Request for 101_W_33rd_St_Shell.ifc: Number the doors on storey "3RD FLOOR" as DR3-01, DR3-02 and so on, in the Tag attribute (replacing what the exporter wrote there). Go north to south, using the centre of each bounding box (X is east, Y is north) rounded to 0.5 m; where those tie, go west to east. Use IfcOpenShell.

First a look at what the model holds.

```python
import ifcopenshell
import ifcopenshell.util.element
import ifcopenshell.util.placement

model = ifcopenshell.open("101_W_33rd_St_Shell.ifc")
print(model.schema)
storey = next(s for s in model.by_type("IfcBuildingStorey") if s.Name == "3RD FLOOR")
doors = [e for e in ifcopenshell.util.element.get_decomposition(storey) if e.is_a("IfcDoor")]
for e in sorted(doors, key=lambda e: e.id()):
    origin = ifcopenshell.util.placement.get_local_placement(e.ObjectPlacement)[:3, 3]
    print(e.id(), e.Tag, e.Name, origin.round(2) + 0.0, sep=" | ")
```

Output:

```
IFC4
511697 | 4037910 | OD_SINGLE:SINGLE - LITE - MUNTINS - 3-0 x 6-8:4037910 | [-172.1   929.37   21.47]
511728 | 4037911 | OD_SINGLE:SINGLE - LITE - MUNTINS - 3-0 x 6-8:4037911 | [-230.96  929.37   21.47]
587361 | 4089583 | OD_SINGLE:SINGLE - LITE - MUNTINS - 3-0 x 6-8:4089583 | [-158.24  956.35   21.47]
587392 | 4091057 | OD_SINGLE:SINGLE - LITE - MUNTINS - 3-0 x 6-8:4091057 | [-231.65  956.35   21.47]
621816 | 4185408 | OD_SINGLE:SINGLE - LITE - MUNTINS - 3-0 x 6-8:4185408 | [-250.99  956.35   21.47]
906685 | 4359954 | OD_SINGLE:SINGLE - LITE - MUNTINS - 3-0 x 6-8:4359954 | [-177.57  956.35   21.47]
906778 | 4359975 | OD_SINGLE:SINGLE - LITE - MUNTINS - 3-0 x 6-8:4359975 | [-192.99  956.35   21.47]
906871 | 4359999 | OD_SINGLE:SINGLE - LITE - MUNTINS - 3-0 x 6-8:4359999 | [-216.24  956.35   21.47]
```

```python
import ifcopenshell
import ifcopenshell.geom
import ifcopenshell.util.element
import ifcopenshell.util.shape

model = ifcopenshell.open("101_W_33rd_St_Shell.ifc")
settings = ifcopenshell.geom.settings()
settings.set("use-world-coords", True)


def centre(element):
    shape = ifcopenshell.geom.create_shape(settings, element)
    return ifcopenshell.util.shape.get_bbox_centroid(shape.geometry)


storey = next(s for s in model.by_type("IfcBuildingStorey") if s.Name == "3RD FLOOR")
doors = [e for e in ifcopenshell.util.element.get_decomposition(storey) if e.is_a("IfcDoor")]

# Insertion points can sit at a corner or the storey origin, so sort by the geometry (in metres).
centres = {e: centre(e) for e in doors}
doors.sort(key=lambda e: (-round(centres[e][1] / 0.5), centres[e][0]))

for i, e in enumerate(doors, start=1):
    number = f"DR3-{i:02d}"
    e.Tag = number
    print(e.id(), number)

model.write("101_W_33rd_St_Shell_edited.ifc")
```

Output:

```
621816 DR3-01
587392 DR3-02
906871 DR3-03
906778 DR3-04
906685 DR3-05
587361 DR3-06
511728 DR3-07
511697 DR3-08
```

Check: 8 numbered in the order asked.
